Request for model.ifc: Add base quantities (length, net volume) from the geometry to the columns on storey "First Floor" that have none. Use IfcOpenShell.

First a look at what the model holds.

```python
import ifcopenshell
import ifcopenshell.util.element
import ifcopenshell.util.unit

model = ifcopenshell.open("model.ifc")
print(model.schema)
for unit_type in ("LENGTHUNIT", "AREAUNIT", "VOLUMEUNIT"):
    print(unit_type, ifcopenshell.util.unit.calculate_unit_scale(model, unit_type))
storey = next(s for s in model.by_type("IfcBuildingStorey") if s.Name == "First Floor")
columns = [e for e in ifcopenshell.util.element.get_decomposition(storey) if e.is_a("IfcColumn")]
for e in sorted(columns, key=lambda e: e.id()):
    print(e.id(), e.is_a(), e.Name, list(ifcopenshell.util.element.get_psets(e, qtos_only=True)), sep=" | ")
```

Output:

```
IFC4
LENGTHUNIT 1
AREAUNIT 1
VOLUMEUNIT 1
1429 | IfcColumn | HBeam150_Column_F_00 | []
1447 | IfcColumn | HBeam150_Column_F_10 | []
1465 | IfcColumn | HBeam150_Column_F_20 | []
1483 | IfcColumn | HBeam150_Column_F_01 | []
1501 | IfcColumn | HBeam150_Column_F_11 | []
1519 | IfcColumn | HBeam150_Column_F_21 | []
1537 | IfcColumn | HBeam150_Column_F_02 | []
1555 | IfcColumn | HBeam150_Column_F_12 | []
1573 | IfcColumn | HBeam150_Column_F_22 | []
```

```python
import ifcopenshell
import ifcopenshell.api.pset
import ifcopenshell.geom
import ifcopenshell.util.element
import ifcopenshell.util.shape
import ifcopenshell.util.unit

model = ifcopenshell.open("model.ifc")
unit_scale = ifcopenshell.util.unit.calculate_unit_scale(model)
volume_scale = ifcopenshell.util.unit.calculate_unit_scale(model, "VOLUMEUNIT")
settings = ifcopenshell.geom.settings()

storey = next(s for s in model.by_type("IfcBuildingStorey") if s.Name == "First Floor")
columns = [e for e in ifcopenshell.util.element.get_decomposition(storey) if e.is_a("IfcColumn")]

for e in sorted(columns, key=lambda e: e.id()):
    if ifcopenshell.util.element.get_psets(e, qtos_only=True, should_inherit=False):
        continue
    # Geometry comes back in metres, in the element's own axes.
    shape = ifcopenshell.geom.create_shape(settings, e)
    values = {
        "Length": ifcopenshell.util.shape.get_z(shape.geometry) / unit_scale,
        "NetVolume": ifcopenshell.util.shape.get_volume(shape.geometry) / volume_scale,
    }
    qto = ifcopenshell.api.pset.add_qto(model, product=e, name="Qto_ColumnBaseQuantities")
    ifcopenshell.api.pset.edit_qto(model, qto=qto, properties=values)
    print(e.id(), {k: round(v, 3) for k, v in values.items()})

model.write("model_v2.ifc")
```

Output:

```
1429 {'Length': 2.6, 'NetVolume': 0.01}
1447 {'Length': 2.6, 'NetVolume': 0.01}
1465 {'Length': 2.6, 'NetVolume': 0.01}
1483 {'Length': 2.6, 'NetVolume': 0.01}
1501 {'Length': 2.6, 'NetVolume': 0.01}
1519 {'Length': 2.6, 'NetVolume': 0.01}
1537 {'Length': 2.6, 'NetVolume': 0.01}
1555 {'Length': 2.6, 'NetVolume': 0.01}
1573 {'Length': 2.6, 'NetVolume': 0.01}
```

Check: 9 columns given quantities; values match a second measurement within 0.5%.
